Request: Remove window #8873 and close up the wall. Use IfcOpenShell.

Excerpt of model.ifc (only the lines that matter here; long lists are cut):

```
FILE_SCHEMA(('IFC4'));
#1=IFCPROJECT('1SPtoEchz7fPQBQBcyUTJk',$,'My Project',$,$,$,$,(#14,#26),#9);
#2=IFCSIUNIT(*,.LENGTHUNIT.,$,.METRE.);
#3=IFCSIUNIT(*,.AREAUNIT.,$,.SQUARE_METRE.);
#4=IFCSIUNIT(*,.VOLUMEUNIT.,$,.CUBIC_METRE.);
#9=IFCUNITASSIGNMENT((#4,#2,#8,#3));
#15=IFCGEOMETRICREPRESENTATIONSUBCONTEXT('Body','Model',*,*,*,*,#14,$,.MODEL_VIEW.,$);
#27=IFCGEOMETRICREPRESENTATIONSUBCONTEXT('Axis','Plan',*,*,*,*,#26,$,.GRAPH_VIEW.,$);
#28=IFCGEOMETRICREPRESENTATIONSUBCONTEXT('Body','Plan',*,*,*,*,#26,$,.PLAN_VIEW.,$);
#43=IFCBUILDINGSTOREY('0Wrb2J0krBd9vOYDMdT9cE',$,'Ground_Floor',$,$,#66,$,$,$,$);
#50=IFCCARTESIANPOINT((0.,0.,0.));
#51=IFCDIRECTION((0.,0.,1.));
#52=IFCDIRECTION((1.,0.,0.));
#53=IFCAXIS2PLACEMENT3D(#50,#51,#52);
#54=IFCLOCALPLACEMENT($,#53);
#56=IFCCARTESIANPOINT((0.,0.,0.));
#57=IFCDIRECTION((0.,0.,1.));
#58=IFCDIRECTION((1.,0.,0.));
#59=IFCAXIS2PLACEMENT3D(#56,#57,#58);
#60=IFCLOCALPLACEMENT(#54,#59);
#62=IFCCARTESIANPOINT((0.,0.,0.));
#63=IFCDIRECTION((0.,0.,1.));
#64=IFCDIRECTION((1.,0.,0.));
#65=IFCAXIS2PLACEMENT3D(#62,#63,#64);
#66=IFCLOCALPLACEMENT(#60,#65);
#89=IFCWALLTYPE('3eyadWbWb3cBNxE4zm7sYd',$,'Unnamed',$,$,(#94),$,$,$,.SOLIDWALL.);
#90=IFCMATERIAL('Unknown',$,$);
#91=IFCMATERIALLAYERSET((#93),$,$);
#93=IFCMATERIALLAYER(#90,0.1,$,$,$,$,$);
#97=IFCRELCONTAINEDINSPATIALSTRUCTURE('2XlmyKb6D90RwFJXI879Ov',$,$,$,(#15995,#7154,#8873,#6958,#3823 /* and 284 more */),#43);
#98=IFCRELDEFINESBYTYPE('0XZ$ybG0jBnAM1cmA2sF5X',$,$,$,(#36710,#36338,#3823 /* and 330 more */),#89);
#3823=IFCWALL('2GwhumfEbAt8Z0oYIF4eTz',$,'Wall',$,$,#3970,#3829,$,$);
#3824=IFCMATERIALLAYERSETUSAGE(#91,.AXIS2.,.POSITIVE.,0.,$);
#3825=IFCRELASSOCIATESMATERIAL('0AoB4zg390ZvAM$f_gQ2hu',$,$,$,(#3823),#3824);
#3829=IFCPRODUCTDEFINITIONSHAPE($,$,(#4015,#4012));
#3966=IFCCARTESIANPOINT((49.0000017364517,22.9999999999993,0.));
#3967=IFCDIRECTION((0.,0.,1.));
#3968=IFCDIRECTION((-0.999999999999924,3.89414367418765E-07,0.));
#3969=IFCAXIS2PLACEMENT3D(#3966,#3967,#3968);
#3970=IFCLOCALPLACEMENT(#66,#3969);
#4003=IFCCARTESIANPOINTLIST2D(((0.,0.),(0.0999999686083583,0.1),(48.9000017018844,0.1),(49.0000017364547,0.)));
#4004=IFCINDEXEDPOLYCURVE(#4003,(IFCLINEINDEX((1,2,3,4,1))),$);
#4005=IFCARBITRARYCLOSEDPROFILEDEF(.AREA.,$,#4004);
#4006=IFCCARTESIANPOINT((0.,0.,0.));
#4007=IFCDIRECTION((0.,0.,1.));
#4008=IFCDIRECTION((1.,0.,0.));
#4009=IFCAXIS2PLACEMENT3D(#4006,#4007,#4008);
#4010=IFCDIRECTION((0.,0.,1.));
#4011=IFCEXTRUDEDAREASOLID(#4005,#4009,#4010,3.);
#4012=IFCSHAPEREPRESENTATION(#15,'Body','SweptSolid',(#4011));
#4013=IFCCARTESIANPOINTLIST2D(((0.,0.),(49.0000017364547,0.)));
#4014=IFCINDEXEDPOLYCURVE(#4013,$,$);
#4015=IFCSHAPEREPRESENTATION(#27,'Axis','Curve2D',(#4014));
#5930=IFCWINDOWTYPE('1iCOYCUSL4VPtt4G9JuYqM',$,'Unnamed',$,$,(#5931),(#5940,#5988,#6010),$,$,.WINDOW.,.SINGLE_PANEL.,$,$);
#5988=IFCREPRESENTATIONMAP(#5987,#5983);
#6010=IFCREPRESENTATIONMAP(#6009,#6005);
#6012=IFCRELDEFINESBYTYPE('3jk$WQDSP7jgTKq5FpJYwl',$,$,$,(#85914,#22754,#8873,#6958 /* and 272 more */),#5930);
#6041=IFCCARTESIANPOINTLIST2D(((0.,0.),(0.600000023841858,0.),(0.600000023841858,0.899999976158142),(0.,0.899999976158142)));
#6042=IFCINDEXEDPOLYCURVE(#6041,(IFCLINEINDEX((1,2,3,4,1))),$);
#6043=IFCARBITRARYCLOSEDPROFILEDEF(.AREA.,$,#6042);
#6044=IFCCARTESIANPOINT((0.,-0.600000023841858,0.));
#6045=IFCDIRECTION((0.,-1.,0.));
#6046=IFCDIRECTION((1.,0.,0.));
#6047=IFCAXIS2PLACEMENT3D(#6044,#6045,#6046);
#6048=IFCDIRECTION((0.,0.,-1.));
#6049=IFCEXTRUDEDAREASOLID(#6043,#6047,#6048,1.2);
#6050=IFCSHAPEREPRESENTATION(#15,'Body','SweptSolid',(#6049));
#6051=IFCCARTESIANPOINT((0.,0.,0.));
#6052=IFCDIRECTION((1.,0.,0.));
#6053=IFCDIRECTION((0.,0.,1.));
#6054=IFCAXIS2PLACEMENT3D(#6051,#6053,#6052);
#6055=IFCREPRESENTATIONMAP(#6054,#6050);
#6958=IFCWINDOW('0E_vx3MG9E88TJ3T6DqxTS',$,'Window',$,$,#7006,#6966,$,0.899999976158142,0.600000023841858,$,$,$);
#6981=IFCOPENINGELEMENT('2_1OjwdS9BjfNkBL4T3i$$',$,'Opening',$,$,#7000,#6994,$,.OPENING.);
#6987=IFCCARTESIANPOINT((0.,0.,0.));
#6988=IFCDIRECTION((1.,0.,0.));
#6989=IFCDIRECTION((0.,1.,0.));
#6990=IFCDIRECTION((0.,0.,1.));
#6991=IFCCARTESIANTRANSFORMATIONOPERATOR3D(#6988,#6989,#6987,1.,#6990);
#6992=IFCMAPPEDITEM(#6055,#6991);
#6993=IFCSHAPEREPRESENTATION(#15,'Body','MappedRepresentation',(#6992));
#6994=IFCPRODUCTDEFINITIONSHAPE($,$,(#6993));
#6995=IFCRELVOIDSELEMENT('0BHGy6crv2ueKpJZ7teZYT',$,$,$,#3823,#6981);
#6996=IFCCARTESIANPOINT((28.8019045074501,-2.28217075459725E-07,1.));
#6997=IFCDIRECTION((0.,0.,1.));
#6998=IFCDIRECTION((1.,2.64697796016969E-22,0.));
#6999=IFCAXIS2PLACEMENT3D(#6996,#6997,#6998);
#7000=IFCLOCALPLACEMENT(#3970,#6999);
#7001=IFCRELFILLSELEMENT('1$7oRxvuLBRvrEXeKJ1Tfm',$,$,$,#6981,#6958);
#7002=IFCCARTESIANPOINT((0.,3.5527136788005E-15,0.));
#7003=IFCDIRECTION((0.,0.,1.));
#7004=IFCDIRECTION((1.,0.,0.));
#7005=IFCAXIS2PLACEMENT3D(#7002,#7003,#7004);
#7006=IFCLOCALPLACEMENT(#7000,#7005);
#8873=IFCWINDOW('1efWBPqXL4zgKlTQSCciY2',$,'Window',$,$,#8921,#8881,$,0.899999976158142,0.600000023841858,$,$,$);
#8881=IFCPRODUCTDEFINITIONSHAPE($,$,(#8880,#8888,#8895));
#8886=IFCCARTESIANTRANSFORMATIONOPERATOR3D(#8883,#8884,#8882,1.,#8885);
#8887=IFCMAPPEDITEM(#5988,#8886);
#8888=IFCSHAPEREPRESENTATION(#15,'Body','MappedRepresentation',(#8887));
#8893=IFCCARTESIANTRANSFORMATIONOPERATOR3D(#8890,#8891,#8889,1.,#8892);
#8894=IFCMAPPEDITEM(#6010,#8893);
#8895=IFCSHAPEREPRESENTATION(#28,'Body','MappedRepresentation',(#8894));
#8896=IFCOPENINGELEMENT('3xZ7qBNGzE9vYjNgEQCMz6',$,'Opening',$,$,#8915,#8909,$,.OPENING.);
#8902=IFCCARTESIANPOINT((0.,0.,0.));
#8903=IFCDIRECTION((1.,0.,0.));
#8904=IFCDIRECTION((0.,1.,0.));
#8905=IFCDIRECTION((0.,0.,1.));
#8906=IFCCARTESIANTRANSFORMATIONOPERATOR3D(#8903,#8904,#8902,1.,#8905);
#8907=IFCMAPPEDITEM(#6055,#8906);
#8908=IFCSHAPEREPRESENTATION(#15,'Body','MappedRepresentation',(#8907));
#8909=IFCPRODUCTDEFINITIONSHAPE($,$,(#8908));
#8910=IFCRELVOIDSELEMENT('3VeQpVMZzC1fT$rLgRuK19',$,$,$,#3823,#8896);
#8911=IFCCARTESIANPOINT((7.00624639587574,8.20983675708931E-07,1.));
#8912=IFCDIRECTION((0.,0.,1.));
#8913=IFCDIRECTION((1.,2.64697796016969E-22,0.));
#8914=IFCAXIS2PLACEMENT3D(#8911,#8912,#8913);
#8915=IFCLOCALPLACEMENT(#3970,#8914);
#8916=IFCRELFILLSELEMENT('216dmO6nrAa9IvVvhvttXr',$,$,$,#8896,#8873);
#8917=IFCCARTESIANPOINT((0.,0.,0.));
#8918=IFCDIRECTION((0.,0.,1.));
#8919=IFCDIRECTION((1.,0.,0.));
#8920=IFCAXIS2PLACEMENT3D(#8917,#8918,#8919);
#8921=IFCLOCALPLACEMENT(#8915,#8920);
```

```python
import ifcopenshell
import ifcopenshell.api.feature
import ifcopenshell.api.root
import ifcopenshell.geom
import ifcopenshell.util.shape

model = ifcopenshell.open("model.ifc")
settings = ifcopenshell.geom.settings()


def volume(element):
    """Net volume in cubic metres, openings subtracted."""
    shape = ifcopenshell.geom.create_shape(settings, element)
    return ifcopenshell.util.shape.get_volume(shape.geometry)


window = model.by_id(8873)
opening = window.FillsVoids[0].RelatingOpeningElement
wall = opening.VoidsElements[0].RelatingBuildingElement
before = volume(wall)

ifcopenshell.api.root.remove_product(model, product=window)
ifcopenshell.api.feature.remove_feature(model, feature=opening)

after = volume(wall)

print(f"wall volume {before:.3f} -> {after:.3f} m3")

model.write("model_rev.ifc")
```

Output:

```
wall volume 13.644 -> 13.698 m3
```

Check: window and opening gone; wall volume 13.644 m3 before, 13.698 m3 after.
